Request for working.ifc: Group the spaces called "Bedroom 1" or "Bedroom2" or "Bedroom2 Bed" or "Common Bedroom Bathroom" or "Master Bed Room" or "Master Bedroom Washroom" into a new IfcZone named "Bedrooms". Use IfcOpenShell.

First a look at what the model holds.

```python
import ifcopenshell

model = ifcopenshell.open("working.ifc")
print(model.schema)
seen = {}
for space in model.by_type("IfcSpace"):
    seen[space.Name] = seen.get(space.Name, 0) + 1
for name, count in sorted(seen.items(), key=str):
    print(count, "x", name)
print("zones:", [z.Name for z in model.by_type("IfcZone")][:20])
```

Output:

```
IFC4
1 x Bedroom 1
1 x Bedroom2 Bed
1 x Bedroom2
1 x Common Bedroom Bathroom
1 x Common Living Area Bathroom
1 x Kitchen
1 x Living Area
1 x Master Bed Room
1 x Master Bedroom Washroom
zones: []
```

```python
import ifcopenshell
import ifcopenshell.api.group
import ifcopenshell.api.root

model = ifcopenshell.open("working.ifc")

names = {"Bedroom 1", "Bedroom2", "Bedroom2 Bed", "Common Bedroom Bathroom", "Master Bed Room", "Master Bedroom Washroom"}
spaces = [s for s in model.by_type("IfcSpace") if s.Name in names]

zone = ifcopenshell.api.root.create_entity(model, ifc_class="IfcZone", name="Bedrooms")
ifcopenshell.api.group.assign_group(model, products=spaces, group=zone)
print(len(spaces), "spaces in", zone.Name)

model.write("working_updated.ifc")
```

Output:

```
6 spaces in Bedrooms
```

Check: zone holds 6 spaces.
